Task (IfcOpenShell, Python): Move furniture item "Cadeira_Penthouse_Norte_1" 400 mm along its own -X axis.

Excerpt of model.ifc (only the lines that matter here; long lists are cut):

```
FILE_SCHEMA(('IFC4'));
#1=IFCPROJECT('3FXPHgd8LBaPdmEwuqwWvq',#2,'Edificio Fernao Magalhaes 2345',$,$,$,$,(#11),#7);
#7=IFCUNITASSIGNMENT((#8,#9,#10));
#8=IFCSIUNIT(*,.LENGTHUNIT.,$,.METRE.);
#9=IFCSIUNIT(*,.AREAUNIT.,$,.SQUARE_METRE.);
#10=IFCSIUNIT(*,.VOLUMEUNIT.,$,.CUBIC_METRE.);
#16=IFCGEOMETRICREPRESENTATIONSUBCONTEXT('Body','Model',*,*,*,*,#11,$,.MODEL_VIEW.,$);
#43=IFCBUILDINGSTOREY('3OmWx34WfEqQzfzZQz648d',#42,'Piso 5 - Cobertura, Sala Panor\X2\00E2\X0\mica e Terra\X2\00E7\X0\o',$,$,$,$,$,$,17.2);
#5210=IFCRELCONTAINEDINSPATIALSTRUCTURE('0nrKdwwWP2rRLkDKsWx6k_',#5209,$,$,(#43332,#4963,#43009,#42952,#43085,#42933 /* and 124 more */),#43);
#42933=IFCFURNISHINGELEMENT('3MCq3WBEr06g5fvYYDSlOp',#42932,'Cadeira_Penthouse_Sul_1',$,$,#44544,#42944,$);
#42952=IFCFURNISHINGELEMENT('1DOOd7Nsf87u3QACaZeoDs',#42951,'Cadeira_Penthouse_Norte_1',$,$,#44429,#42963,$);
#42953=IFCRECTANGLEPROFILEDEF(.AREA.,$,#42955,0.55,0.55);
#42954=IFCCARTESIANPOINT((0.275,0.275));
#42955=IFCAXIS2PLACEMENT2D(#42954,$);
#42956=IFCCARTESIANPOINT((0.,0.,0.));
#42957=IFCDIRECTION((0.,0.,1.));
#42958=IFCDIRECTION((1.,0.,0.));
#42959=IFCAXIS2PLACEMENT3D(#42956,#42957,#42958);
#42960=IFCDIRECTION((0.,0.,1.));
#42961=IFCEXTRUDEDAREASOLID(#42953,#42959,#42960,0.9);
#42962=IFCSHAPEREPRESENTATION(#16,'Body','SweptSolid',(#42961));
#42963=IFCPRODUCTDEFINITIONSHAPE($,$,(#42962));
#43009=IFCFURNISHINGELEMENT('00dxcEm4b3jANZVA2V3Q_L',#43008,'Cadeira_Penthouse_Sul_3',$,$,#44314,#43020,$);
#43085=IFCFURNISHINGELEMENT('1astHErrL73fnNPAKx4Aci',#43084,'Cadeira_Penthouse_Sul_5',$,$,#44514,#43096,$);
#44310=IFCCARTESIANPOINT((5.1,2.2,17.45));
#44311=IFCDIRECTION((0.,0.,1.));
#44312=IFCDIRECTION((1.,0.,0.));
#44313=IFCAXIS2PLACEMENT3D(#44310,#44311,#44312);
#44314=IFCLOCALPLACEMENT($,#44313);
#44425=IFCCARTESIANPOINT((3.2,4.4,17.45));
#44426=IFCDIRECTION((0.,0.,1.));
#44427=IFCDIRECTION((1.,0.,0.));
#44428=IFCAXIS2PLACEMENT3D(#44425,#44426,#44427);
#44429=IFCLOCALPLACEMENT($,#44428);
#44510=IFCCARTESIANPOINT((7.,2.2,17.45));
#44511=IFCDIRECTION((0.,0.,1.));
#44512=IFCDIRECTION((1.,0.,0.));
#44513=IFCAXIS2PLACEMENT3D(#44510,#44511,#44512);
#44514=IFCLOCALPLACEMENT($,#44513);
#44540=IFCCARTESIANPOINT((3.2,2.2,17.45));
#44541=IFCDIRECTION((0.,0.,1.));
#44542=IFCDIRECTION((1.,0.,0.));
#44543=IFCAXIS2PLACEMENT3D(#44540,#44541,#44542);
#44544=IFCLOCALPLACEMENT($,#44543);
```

```python
import ifcopenshell
import ifcopenshell.api.geometry
import ifcopenshell.util.placement

model = ifcopenshell.open("model.ifc")

item = model.by_guid("1DOOd7Nsf87u3QACaZeoDs")
matrix = ifcopenshell.util.placement.get_local_placement(item.ObjectPlacement)
matrix[:3, 3] -= matrix[:3, 0] * 0.4
ifcopenshell.api.geometry.edit_object_placement(model, product=item, matrix=matrix, is_si=False)

print(ifcopenshell.util.placement.get_local_placement(item.ObjectPlacement).round(3) + 0.0)

model.write("model_v2.ifc")
```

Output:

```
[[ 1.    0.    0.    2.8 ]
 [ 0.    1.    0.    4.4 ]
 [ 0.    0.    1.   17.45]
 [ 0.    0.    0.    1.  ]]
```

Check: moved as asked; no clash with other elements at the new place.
